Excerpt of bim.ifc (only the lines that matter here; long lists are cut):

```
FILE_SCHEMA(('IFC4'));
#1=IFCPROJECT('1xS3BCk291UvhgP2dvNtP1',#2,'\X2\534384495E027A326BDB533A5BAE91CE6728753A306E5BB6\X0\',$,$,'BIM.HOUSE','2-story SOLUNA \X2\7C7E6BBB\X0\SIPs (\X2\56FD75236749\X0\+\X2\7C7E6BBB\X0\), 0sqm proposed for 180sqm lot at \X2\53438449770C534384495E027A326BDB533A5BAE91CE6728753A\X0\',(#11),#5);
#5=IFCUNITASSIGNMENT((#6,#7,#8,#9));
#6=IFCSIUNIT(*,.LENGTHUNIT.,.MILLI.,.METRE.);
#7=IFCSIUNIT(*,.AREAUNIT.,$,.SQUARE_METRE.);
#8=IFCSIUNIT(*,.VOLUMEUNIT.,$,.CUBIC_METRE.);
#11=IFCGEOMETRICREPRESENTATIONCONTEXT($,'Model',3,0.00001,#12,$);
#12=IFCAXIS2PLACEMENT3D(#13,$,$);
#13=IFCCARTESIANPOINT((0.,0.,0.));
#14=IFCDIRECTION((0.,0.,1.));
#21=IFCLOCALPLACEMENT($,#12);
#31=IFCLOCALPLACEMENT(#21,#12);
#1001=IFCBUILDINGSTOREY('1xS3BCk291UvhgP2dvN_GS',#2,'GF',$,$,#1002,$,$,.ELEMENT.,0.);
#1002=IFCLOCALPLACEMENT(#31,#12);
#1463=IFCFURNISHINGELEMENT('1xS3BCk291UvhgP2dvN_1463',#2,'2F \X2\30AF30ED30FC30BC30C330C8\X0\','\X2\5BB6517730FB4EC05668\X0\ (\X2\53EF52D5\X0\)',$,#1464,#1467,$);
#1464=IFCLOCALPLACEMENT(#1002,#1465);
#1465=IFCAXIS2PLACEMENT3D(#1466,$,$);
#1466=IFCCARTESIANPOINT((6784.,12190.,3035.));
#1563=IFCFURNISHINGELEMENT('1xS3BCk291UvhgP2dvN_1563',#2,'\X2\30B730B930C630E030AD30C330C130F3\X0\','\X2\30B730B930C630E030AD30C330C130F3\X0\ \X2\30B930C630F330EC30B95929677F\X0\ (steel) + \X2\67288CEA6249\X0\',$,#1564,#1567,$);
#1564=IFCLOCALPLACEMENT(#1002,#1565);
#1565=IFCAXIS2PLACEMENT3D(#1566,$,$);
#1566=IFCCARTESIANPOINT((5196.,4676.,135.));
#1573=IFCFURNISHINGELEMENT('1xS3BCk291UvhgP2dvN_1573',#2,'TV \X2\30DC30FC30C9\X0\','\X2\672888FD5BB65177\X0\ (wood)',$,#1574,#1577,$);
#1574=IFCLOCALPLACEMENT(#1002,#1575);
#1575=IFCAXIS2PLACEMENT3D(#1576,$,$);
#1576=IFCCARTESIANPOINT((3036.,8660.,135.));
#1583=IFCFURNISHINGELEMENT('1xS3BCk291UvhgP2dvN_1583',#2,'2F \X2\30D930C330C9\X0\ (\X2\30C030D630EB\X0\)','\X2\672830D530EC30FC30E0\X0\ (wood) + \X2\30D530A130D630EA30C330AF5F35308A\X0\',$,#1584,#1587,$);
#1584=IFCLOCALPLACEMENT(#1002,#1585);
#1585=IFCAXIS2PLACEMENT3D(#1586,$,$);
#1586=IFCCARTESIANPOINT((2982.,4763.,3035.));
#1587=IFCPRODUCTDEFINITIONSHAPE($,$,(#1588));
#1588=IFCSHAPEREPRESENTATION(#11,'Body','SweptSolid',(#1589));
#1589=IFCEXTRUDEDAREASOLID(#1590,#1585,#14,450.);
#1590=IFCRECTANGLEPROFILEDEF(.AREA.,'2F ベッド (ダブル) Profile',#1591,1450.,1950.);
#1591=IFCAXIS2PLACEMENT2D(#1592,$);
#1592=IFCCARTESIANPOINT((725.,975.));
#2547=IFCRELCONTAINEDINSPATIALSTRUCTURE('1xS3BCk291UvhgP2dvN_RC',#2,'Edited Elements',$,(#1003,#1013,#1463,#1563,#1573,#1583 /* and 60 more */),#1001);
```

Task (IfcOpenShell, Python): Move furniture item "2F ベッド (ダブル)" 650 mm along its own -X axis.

```python
import ifcopenshell
import ifcopenshell.api.geometry
import ifcopenshell.util.placement

model = ifcopenshell.open("bim.ifc")

item = model.by_id(1583)
matrix = ifcopenshell.util.placement.get_local_placement(item.ObjectPlacement)
matrix[:3, 3] -= matrix[:3, 0] * 650.0
ifcopenshell.api.geometry.edit_object_placement(model, product=item, matrix=matrix, is_si=False)

print(ifcopenshell.util.placement.get_local_placement(item.ObjectPlacement).round(3) + 0.0)

model.write("bim_v2.ifc")
```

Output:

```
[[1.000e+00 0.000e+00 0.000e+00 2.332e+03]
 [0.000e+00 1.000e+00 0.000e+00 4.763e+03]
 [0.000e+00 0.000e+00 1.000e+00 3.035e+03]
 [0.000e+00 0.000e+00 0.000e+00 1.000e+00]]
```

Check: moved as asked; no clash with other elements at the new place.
